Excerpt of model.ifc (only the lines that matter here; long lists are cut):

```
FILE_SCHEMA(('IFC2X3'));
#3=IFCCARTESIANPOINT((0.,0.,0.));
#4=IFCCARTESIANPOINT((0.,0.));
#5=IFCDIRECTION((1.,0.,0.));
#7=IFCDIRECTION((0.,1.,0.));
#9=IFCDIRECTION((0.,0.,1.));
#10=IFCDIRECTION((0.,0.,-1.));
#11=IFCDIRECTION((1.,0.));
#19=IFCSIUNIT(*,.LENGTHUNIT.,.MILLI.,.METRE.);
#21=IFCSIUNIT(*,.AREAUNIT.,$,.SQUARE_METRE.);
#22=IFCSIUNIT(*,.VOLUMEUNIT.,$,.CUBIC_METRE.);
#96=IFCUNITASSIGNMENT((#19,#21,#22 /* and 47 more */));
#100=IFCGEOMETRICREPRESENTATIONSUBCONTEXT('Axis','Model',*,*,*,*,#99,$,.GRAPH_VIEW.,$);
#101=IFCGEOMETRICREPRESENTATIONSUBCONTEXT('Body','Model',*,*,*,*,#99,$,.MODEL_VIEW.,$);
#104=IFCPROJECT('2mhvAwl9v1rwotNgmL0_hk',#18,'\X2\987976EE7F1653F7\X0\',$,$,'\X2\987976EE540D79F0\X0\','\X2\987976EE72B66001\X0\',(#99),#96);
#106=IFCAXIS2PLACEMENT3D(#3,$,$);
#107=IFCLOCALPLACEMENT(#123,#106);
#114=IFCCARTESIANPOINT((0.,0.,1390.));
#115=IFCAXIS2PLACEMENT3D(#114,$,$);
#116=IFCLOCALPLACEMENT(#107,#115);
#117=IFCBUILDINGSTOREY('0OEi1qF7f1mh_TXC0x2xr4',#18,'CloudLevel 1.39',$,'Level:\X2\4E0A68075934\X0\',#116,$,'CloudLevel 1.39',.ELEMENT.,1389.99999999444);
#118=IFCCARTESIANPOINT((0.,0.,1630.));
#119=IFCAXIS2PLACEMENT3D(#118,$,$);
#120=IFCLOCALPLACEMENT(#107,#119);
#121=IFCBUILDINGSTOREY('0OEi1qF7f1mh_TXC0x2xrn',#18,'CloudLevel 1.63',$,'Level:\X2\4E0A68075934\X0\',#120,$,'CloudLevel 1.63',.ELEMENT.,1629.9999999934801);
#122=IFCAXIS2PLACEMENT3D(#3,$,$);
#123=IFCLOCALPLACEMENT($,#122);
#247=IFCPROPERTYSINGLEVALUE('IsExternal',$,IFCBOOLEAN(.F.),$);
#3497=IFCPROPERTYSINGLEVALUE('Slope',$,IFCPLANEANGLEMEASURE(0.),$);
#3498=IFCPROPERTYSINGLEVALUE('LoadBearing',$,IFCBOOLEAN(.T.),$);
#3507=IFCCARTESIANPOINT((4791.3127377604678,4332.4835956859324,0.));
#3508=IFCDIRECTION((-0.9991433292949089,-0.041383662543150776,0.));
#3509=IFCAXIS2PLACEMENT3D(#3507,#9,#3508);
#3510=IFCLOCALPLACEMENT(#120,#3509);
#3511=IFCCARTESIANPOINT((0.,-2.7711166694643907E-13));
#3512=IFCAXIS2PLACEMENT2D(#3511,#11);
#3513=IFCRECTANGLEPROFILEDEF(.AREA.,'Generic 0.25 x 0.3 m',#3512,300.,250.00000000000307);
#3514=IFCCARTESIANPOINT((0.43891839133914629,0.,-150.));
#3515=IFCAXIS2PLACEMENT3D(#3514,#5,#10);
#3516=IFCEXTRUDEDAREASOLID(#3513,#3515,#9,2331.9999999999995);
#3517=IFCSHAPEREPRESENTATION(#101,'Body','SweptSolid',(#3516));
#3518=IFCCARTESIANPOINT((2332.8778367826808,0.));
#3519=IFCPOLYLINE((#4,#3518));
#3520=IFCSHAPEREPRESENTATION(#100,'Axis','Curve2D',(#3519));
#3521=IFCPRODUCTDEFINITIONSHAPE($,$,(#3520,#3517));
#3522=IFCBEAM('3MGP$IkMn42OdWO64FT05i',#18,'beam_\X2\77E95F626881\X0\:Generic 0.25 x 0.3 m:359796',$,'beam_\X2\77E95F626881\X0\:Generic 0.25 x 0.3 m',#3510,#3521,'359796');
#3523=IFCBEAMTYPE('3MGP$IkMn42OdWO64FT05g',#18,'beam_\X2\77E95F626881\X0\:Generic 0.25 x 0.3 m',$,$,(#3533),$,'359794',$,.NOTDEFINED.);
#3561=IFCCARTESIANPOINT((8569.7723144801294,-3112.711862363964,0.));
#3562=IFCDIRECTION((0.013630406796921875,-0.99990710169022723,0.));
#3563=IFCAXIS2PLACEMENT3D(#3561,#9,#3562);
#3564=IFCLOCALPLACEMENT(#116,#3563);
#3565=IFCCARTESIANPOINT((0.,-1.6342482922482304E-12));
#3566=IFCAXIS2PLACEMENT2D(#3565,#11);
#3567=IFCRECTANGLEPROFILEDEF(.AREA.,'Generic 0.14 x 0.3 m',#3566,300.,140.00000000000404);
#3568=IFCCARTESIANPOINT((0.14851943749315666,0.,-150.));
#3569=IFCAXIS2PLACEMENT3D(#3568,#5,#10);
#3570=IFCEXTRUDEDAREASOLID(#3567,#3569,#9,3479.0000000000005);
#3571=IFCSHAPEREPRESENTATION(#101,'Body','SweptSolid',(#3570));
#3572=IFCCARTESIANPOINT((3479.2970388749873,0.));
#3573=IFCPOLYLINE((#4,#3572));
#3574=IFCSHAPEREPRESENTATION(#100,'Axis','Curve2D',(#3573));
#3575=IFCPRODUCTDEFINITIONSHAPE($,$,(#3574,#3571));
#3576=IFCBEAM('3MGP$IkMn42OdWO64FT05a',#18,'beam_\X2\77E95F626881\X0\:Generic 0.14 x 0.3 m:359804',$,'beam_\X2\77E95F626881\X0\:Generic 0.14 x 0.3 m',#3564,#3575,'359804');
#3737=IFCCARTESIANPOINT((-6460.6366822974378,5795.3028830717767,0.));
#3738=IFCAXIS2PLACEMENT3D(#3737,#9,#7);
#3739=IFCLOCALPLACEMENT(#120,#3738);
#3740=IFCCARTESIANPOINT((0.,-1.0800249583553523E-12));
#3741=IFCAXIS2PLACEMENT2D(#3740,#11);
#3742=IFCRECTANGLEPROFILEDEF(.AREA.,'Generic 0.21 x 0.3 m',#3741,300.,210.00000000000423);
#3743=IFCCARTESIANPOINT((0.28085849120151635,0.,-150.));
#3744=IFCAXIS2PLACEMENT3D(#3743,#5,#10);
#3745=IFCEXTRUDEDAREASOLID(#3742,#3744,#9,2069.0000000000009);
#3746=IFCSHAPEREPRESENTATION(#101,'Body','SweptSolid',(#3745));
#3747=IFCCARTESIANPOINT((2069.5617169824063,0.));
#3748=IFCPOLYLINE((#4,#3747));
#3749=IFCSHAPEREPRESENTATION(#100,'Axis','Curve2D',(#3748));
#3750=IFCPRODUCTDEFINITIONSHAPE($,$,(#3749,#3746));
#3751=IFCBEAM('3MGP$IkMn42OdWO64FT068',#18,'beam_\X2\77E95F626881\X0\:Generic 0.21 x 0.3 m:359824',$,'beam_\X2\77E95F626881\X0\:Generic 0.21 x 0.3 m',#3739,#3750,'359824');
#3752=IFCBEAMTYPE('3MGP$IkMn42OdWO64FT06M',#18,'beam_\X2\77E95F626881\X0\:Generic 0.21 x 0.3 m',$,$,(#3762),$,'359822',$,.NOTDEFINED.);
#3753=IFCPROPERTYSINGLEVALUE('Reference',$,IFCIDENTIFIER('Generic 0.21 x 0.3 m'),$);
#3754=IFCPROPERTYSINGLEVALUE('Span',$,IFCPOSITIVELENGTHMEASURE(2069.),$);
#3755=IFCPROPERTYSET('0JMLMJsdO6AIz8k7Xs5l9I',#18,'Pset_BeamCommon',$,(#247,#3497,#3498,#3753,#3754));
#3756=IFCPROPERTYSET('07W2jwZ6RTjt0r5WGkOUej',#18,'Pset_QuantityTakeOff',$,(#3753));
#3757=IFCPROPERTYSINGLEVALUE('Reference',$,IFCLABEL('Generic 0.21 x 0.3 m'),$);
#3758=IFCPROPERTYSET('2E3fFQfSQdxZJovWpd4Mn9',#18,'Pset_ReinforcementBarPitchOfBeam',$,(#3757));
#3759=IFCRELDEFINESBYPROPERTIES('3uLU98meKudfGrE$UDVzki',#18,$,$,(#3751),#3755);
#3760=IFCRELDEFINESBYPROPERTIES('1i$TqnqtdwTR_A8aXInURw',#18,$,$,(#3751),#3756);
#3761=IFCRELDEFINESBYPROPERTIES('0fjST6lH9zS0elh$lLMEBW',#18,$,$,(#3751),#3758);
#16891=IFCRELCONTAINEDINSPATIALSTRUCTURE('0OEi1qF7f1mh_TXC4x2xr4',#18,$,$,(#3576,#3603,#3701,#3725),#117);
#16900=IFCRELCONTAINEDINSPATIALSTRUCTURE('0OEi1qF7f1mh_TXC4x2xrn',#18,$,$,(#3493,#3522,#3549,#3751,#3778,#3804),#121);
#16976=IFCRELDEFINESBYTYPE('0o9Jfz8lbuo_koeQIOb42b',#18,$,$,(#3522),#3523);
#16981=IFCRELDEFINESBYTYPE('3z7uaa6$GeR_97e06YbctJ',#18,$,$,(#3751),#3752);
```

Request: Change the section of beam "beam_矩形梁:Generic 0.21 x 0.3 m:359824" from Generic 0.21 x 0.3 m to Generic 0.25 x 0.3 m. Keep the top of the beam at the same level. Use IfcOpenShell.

```python
import ifcopenshell
import ifcopenshell.api.pset
import ifcopenshell.api.type
import ifcopenshell.util.element
import ifcopenshell.util.representation

model = ifcopenshell.open("model.ifc")

member = model.by_guid("3MGP$IkMn42OdWO64FT068")
source = next(p for p in model.by_type("IfcRectangleProfileDef") if p.ProfileName == "Generic 0.25 x 0.3 m")

body = ifcopenshell.util.representation.get_representation(member, "Model", "Body")
solid = body.Items[0]
old_profile = solid.SweptArea

# Copy the section's sizes but keep this member's own profile position.
profile = ifcopenshell.util.element.copy(model, source)
# Profiles are centred, so shift by half the change in depth to hold the top.
shift = (old_profile.XDim - profile.XDim) / 2
x, y = old_profile.Position.Location.Coordinates
up = (-1.0, 0.0)  # upwards, in the solid's own plane
location = model.createIfcCartesianPoint((x + up[0] * shift, y + up[1] * shift))
profile.Position = model.createIfcAxis2Placement2D(location, old_profile.Position.RefDirection)
solid.SweptArea = profile
if not model.get_total_inverses(old_profile):
    ifcopenshell.util.element.remove_deep2(model, old_profile)

new_type = model.by_guid("3MGP$IkMn42OdWO64FT05g")
ifcopenshell.api.type.assign_type(
    model, related_objects=[member], relating_type=new_type, should_map_representations=False
)
member.Name = member.Name.replace("Generic 0.21 x 0.3 m", "Generic 0.25 x 0.3 m")
member.ObjectType = "beam_矩形梁:Generic 0.25 x 0.3 m"
pset = model.by_id(ifcopenshell.util.element.get_pset(member, "Pset_BeamCommon", should_inherit=False)["id"])
ifcopenshell.api.pset.edit_pset(model, pset=pset, properties={"Reference": "Generic 0.25 x 0.3 m"})
pset = model.by_id(ifcopenshell.util.element.get_pset(member, "Pset_QuantityTakeOff", should_inherit=False)["id"])
ifcopenshell.api.pset.edit_pset(model, pset=pset, properties={"Reference": "Generic 0.25 x 0.3 m"})
pset = model.by_id(ifcopenshell.util.element.get_pset(member, "Pset_ReinforcementBarPitchOfBeam", should_inherit=False)["id"])
ifcopenshell.api.pset.edit_pset(model, pset=pset, properties={"Reference": "Generic 0.25 x 0.3 m"})

print(solid.SweptArea)

model.write("model_updated.ifc")
```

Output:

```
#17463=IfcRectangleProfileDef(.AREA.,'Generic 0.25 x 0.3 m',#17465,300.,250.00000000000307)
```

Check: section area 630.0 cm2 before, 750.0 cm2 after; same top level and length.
